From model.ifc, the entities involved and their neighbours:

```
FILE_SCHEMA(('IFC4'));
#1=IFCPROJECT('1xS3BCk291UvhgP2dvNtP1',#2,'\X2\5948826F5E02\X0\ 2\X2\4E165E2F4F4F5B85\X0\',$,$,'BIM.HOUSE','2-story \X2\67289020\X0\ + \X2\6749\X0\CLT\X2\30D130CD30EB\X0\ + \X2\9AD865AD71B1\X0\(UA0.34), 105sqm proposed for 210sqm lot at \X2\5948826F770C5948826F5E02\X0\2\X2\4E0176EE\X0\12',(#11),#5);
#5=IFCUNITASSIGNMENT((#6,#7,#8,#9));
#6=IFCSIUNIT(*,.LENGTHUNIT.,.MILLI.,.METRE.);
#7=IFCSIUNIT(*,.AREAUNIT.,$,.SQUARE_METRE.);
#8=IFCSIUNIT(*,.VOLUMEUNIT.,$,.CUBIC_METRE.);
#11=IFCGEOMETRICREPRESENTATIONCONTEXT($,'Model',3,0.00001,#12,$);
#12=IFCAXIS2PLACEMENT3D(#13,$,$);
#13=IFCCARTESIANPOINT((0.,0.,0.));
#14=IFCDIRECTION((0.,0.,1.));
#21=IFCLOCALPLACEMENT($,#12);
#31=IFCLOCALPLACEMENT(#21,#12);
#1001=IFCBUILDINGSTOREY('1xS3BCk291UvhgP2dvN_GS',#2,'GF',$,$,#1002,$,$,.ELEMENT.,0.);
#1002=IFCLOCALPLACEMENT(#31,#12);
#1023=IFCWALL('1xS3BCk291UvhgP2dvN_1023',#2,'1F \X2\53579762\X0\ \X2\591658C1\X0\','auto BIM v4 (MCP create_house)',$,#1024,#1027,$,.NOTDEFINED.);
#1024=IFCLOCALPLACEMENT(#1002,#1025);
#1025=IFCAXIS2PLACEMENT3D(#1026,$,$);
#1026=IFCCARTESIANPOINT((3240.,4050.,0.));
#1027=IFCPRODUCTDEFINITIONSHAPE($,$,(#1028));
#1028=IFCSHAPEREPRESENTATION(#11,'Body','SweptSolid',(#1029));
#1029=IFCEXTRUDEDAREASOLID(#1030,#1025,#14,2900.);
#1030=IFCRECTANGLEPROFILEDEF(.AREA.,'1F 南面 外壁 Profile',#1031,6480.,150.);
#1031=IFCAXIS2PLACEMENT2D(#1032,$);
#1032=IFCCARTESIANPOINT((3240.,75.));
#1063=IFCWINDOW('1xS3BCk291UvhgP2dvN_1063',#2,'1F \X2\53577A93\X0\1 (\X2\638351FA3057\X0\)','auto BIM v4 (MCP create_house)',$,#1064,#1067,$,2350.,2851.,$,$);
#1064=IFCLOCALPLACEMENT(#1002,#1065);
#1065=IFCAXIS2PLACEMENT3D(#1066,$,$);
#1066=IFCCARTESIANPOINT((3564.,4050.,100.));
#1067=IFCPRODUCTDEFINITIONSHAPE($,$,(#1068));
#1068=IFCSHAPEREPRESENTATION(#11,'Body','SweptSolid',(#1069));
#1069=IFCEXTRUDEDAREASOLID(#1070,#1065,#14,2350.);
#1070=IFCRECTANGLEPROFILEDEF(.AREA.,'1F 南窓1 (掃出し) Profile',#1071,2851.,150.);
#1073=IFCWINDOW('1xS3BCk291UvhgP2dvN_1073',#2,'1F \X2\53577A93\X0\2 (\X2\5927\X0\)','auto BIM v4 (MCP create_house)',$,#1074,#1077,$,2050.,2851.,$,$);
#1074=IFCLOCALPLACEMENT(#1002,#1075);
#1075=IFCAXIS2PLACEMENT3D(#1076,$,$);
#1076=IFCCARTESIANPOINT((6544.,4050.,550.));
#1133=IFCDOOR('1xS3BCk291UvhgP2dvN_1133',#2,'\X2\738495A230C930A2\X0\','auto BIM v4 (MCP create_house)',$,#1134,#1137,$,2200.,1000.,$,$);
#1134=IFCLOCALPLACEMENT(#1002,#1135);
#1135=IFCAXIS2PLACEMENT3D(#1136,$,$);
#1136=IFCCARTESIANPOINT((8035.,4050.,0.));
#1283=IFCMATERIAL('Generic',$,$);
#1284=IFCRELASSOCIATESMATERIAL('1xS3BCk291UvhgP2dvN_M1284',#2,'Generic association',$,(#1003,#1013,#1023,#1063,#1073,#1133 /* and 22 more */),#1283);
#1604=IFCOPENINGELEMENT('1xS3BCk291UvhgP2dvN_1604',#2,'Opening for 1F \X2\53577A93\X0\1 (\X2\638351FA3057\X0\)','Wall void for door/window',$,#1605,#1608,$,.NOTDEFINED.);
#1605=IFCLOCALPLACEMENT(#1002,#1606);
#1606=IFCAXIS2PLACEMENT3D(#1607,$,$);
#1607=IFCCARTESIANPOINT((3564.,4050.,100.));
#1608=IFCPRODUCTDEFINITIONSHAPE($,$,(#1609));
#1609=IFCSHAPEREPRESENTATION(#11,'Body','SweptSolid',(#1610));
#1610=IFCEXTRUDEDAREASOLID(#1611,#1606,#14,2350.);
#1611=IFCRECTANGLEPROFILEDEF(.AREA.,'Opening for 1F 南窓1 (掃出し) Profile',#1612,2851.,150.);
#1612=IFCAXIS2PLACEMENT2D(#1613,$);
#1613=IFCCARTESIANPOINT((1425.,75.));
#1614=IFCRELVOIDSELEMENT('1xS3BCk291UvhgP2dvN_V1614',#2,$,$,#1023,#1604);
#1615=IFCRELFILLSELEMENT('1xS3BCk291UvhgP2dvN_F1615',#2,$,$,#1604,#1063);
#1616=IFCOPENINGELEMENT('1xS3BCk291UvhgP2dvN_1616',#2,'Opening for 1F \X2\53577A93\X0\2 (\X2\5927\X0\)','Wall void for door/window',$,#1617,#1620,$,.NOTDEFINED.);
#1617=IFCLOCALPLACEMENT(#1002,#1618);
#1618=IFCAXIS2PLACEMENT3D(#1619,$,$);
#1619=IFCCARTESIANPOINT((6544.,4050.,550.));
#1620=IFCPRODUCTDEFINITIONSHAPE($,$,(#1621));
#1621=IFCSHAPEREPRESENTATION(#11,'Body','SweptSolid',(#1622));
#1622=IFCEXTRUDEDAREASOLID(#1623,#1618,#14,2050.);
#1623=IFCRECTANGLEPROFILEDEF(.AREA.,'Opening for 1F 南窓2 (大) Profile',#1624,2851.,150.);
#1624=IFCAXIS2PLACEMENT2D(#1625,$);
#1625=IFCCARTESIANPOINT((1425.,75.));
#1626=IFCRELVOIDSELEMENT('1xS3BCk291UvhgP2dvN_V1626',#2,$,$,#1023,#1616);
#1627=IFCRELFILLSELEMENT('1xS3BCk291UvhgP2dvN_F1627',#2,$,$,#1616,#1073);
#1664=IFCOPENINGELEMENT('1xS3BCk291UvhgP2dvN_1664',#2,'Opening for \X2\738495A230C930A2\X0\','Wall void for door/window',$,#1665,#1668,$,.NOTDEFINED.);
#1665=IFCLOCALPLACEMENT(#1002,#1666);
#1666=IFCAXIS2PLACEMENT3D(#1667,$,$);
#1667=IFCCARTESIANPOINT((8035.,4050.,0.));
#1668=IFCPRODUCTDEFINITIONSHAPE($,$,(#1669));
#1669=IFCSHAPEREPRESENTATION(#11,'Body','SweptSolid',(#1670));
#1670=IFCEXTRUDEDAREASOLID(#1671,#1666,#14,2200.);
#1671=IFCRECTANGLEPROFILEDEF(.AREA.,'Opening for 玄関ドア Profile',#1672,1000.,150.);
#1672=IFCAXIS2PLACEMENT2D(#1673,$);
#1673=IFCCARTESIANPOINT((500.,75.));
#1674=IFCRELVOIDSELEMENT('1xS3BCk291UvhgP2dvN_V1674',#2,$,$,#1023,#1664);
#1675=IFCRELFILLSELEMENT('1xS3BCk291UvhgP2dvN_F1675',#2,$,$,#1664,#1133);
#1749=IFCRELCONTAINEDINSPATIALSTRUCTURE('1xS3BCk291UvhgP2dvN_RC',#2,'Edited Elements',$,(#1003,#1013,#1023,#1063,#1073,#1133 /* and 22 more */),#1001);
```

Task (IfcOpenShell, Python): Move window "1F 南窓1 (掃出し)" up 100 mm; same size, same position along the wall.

```python
import numpy as np
import ifcopenshell
import ifcopenshell.api.geometry
import ifcopenshell.util.placement
import ifcopenshell.util.unit

model = ifcopenshell.open("model.ifc")
unit_scale = ifcopenshell.util.unit.calculate_unit_scale(model)

window = model.by_id(1063)
opening = window.FillsVoids[0].RelatingOpeningElement
dz = 0.1 / unit_scale

shift = np.array([0.0, 0.0, dz])
# The window is not placed relative to its opening, so move both.
for product in (opening, window):
    matrix = ifcopenshell.util.placement.get_local_placement(product.ObjectPlacement)
    matrix[:3, 3] += shift
    ifcopenshell.api.geometry.edit_object_placement(model, product=product, matrix=matrix, is_si=False)

print(f"moved by {dz * unit_scale:+.3f} m")

model.write("model_v2.ifc")
```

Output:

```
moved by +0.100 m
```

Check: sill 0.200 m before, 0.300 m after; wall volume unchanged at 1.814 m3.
